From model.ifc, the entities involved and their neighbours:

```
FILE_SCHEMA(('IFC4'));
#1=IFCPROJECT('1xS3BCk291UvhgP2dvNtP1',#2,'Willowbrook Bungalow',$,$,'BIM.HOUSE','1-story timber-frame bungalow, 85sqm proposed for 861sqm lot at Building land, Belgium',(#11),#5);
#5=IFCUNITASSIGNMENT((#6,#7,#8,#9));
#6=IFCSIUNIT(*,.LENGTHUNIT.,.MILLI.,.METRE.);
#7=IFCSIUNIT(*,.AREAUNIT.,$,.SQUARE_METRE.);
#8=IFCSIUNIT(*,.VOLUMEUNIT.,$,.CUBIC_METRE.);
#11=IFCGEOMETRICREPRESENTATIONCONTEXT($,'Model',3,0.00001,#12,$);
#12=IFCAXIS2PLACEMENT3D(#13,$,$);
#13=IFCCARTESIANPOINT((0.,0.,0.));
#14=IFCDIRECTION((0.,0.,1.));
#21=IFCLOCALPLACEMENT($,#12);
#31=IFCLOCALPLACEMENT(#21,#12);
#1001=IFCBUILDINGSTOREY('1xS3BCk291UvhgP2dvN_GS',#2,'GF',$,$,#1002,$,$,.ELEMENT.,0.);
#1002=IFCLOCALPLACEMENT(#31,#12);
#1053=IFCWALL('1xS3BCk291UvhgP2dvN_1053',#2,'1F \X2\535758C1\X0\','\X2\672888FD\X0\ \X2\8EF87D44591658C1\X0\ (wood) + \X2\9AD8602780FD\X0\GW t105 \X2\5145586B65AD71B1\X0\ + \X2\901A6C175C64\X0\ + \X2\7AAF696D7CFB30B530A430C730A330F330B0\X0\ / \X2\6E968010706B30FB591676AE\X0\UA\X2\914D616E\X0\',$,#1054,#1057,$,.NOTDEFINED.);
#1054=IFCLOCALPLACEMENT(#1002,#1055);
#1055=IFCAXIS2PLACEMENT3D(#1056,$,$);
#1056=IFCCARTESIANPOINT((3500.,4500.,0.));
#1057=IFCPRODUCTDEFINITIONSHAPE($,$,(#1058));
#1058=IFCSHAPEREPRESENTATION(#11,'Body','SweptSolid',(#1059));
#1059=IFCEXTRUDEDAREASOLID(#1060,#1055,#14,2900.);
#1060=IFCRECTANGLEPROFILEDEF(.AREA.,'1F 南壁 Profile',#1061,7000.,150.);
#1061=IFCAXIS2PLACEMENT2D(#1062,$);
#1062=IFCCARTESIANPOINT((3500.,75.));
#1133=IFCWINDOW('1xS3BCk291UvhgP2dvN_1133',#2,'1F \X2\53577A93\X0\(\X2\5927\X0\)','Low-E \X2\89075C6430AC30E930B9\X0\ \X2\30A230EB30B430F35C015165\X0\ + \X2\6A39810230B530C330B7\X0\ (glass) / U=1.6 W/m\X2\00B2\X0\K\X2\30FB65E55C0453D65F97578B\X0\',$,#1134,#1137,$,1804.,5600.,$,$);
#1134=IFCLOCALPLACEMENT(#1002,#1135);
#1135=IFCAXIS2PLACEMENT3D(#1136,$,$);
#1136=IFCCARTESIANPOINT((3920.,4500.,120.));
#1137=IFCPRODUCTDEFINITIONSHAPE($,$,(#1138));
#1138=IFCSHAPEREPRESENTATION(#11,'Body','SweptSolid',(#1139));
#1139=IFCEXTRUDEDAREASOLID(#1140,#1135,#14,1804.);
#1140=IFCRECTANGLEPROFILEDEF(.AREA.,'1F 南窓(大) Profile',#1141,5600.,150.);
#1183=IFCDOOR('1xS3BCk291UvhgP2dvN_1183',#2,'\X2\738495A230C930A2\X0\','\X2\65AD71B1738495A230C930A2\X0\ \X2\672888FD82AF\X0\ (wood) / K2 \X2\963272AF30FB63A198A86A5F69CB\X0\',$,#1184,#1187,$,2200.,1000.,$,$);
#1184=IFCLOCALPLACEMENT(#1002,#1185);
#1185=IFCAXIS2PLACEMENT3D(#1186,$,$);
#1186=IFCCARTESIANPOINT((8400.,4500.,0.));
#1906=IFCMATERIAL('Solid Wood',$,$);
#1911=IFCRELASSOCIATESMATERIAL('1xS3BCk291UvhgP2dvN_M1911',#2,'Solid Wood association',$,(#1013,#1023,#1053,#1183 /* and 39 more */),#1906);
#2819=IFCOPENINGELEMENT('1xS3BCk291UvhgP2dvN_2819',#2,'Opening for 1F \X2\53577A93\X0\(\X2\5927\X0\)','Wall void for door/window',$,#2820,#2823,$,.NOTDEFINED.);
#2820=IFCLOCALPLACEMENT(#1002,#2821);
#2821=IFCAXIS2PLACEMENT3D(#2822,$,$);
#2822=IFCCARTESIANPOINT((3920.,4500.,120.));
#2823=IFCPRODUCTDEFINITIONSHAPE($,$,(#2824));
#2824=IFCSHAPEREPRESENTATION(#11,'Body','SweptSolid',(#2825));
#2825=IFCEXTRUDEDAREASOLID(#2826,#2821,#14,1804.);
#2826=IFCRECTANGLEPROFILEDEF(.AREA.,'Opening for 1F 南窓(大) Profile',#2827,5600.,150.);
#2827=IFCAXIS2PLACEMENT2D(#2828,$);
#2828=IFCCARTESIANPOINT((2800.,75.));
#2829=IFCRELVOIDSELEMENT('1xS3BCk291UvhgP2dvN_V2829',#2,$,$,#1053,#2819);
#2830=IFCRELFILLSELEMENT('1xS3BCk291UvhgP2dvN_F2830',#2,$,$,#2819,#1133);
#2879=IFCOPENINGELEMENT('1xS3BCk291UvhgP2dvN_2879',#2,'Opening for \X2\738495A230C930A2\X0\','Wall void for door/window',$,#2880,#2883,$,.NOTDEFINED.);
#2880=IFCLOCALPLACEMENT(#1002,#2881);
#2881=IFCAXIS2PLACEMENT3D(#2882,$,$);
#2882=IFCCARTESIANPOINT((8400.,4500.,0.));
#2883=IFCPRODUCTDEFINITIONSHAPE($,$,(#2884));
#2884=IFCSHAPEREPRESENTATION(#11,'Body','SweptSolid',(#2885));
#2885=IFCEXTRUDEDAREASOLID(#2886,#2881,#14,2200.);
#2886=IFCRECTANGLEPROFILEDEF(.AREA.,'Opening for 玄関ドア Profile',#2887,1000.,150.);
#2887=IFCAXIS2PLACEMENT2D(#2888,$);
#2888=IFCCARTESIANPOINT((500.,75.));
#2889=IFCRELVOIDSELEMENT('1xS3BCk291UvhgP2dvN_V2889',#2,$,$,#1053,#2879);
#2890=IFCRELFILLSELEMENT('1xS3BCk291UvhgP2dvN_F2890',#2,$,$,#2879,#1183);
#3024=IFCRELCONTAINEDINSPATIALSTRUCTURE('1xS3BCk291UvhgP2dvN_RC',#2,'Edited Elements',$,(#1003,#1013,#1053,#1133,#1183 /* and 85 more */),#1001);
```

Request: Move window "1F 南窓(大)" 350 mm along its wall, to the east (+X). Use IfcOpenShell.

```python
import ifcopenshell
import ifcopenshell.api.geometry
import ifcopenshell.util.placement
import ifcopenshell.util.unit

model = ifcopenshell.open("model.ifc")
unit_scale = ifcopenshell.util.unit.calculate_unit_scale(model)

window = model.by_guid("1xS3BCk291UvhgP2dvN_1133")
opening = window.FillsVoids[0].RelatingOpeningElement
wall = opening.VoidsElements[0].RelatingBuildingElement

wall_matrix = ifcopenshell.util.placement.get_local_placement(wall.ObjectPlacement)
shift = wall_matrix[:3, 0] * 0.35 / unit_scale
before = ifcopenshell.util.placement.get_local_placement(window.ObjectPlacement)[:3, 3].copy()

# The window is not placed relative to its opening, so move both.
for product in (opening, window):
    matrix = ifcopenshell.util.placement.get_local_placement(product.ObjectPlacement)
    matrix[:3, 3] += shift
    ifcopenshell.api.geometry.edit_object_placement(model, product=product, matrix=matrix, is_si=False)

after = ifcopenshell.util.placement.get_local_placement(window.ObjectPlacement)[:3, 3]
print("window moved by", (after - before).round(3) + 0.0)

model.write("model_edited.ifc")
```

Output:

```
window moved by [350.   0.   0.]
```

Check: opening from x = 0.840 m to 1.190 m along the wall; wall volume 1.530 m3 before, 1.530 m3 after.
